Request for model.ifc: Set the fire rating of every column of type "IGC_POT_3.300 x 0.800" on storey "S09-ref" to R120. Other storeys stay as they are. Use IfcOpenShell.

First a look at what the model holds.

```python
import ifcopenshell
import ifcopenshell.util.element

model = ifcopenshell.open("model.ifc")
print(model.schema)
storey = next(s for s in model.by_type("IfcBuildingStorey") if s.Name == "S09-ref")
columns = [e for e in ifcopenshell.util.element.get_decomposition(storey) if e.is_a("IfcColumn")]
seen = {}
for e in columns:
    element_type = ifcopenshell.util.element.get_type(e)
    key = (element_type.Name if element_type != e and element_type else None, ifcopenshell.util.element.get_pset(e, "Pset_ColumnCommon", "FireRating"))
    seen[key] = seen.get(key, 0) + 1
for (name, value), count in sorted(seen.items(), key=str):
    print(count, "x", name, "|", value)
```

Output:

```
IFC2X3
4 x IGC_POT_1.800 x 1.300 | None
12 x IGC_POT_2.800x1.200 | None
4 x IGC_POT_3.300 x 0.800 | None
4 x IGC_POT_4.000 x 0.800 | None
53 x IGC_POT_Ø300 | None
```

```python
import ifcopenshell
import ifcopenshell.api.pset
import ifcopenshell.util.element

model = ifcopenshell.open("model.ifc")

storey = next(s for s in model.by_type("IfcBuildingStorey") if s.Name == "S09-ref")
columns = [e for e in ifcopenshell.util.element.get_decomposition(storey) if e.is_a("IfcColumn")]

count = 0
for e in columns:
    element_type = ifcopenshell.util.element.get_type(e)
    if element_type in (None, e) or element_type.Name != "IGC_POT_3.300 x 0.800":
        continue
    # add_pset returns the element's existing set when there is one.
    pset = ifcopenshell.api.pset.add_pset(model, product=e, name="Pset_ColumnCommon")
    ifcopenshell.api.pset.edit_pset(model, pset=pset, properties={"FireRating": "R120"})
    count += 1

print(count, "columns updated")

model.write("model_edited.ifc")
```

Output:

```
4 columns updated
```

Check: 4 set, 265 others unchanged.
